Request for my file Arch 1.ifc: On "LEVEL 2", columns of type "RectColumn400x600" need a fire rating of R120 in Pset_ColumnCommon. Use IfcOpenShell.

First a look at what the model holds.

```python
import ifcopenshell
import ifcopenshell.util.element

model = ifcopenshell.open("my file Arch 1.ifc")
print(model.schema)
storey = next(s for s in model.by_type("IfcBuildingStorey") if s.Name == "LEVEL 2")
columns = [e for e in ifcopenshell.util.element.get_decomposition(storey) if e.is_a("IfcColumn")]
seen = {}
for e in columns:
    element_type = ifcopenshell.util.element.get_type(e)
    key = (element_type.Name if element_type != e and element_type else None, ifcopenshell.util.element.get_pset(e, "Pset_ColumnCommon", "FireRating"))
    seen[key] = seen.get(key, 0) + 1
for (name, value), count in sorted(seen.items(), key=str):
    print(count, "x", name, "|", value)
```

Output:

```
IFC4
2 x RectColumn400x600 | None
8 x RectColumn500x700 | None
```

```python
import ifcopenshell
import ifcopenshell.api.pset
import ifcopenshell.util.element

model = ifcopenshell.open("my file Arch 1.ifc")

storey = next(s for s in model.by_type("IfcBuildingStorey") if s.Name == "LEVEL 2")
columns = [e for e in ifcopenshell.util.element.get_decomposition(storey) if e.is_a("IfcColumn")]

count = 0
for e in columns:
    element_type = ifcopenshell.util.element.get_type(e)
    if element_type in (None, e) or element_type.Name != "RectColumn400x600":
        continue
    # add_pset returns the element's existing set when there is one.
    pset = ifcopenshell.api.pset.add_pset(model, product=e, name="Pset_ColumnCommon")
    ifcopenshell.api.pset.edit_pset(model, pset=pset, properties={"FireRating": "R120"})
    count += 1

print(count, "columns updated")

model.write("my file Arch 1-out.ifc")
```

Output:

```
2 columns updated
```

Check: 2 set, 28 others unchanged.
